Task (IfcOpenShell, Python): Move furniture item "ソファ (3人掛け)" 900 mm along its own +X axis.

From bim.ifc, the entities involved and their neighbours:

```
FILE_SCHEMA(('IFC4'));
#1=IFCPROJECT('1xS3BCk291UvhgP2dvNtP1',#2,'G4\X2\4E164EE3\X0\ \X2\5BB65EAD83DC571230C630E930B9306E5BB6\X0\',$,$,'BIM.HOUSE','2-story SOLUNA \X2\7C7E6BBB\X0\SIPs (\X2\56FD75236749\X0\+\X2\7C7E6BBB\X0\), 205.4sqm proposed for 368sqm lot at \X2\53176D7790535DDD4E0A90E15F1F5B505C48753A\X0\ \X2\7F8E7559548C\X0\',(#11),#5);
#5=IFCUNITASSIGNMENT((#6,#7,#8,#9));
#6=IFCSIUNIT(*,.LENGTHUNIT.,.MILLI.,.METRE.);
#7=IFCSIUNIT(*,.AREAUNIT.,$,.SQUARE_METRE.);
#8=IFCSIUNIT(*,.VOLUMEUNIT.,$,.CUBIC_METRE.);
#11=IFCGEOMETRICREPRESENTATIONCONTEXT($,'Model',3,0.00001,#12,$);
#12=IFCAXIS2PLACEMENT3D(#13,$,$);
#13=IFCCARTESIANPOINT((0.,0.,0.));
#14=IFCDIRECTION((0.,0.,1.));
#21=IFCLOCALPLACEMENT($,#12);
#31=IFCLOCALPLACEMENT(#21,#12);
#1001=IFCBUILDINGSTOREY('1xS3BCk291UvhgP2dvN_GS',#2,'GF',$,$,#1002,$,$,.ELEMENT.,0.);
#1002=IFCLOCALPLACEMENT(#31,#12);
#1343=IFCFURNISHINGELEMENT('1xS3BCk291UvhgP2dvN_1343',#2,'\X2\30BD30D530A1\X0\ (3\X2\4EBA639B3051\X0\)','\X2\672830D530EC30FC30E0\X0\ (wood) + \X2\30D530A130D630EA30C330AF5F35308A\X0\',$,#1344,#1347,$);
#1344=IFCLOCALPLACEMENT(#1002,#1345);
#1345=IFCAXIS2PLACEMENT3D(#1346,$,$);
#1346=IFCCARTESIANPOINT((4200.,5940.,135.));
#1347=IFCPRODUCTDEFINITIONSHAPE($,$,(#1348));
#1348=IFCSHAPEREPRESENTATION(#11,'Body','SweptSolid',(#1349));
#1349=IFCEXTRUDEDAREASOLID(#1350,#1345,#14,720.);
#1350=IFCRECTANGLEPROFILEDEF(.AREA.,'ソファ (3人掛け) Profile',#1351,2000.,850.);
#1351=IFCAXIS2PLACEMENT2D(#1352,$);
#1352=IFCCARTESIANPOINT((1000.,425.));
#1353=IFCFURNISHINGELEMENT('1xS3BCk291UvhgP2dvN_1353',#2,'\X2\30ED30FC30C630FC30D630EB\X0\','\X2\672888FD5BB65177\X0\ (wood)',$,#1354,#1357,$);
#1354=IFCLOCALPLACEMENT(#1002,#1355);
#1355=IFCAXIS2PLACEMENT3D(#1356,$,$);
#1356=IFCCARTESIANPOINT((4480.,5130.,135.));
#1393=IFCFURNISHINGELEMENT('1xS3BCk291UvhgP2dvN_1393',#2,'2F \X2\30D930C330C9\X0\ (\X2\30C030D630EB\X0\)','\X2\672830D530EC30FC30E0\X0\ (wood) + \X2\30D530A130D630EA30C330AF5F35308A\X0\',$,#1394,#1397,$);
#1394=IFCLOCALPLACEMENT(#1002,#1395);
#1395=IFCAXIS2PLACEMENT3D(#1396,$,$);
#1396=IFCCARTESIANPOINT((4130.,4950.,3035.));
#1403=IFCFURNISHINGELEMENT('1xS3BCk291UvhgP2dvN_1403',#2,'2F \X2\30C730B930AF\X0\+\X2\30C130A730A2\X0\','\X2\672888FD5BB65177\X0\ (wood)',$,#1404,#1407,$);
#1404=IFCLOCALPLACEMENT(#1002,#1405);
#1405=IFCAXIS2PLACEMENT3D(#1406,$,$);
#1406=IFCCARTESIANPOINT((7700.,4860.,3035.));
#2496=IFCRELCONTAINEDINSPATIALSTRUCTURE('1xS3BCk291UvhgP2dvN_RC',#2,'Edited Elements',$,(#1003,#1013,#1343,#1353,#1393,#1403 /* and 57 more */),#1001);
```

```python
import ifcopenshell
import ifcopenshell.api.geometry
import ifcopenshell.util.placement
import ifcopenshell.util.unit

model = ifcopenshell.open("bim.ifc")
unit_scale = ifcopenshell.util.unit.calculate_unit_scale(model)

item = model.by_id(1343)
matrix = ifcopenshell.util.placement.get_local_placement(item.ObjectPlacement)
matrix[:3, 3] += matrix[:3, 0] * 0.9 / unit_scale
ifcopenshell.api.geometry.edit_object_placement(model, product=item, matrix=matrix, is_si=False)

print(ifcopenshell.util.placement.get_local_placement(item.ObjectPlacement).round(3) + 0.0)

model.write("bim_edited.ifc")
```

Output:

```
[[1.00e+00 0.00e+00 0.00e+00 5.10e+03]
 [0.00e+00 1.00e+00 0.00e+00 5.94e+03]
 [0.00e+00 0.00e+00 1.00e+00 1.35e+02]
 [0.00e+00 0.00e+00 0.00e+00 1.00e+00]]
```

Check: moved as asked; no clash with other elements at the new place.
